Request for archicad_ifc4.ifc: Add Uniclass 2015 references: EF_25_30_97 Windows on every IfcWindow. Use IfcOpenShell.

First a look at what the model holds.

```python
import ifcopenshell

model = ifcopenshell.open("archicad_ifc4.ifc")
print(model.schema)
print("classifications:", [c.Name for c in model.by_type("IfcClassification")])
for ifc_class in ("IfcDoor", "IfcRoof", "IfcStair", "IfcWall", "IfcWindow"):
    print(ifc_class, len(model.by_type(ifc_class)))
```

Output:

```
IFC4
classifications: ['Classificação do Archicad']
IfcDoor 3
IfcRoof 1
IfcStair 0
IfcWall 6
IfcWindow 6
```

```python
import ifcopenshell
import ifcopenshell.api.classification

model = ifcopenshell.open("archicad_ifc4.ifc")

system = ifcopenshell.api.classification.add_classification(model, classification="Uniclass 2015")

codes = {
    "IfcWindow": ("EF_25_30_97", "Windows"),
}
for ifc_class, (code, name) in codes.items():
    products = model.by_type(ifc_class)
    ifcopenshell.api.classification.add_reference(
        model, products=products, classification=system, identification=code, name=name
    )
    print(code, len(products))

model.write("archicad_ifc4-out.ifc")
```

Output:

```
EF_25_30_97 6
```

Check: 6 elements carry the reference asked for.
